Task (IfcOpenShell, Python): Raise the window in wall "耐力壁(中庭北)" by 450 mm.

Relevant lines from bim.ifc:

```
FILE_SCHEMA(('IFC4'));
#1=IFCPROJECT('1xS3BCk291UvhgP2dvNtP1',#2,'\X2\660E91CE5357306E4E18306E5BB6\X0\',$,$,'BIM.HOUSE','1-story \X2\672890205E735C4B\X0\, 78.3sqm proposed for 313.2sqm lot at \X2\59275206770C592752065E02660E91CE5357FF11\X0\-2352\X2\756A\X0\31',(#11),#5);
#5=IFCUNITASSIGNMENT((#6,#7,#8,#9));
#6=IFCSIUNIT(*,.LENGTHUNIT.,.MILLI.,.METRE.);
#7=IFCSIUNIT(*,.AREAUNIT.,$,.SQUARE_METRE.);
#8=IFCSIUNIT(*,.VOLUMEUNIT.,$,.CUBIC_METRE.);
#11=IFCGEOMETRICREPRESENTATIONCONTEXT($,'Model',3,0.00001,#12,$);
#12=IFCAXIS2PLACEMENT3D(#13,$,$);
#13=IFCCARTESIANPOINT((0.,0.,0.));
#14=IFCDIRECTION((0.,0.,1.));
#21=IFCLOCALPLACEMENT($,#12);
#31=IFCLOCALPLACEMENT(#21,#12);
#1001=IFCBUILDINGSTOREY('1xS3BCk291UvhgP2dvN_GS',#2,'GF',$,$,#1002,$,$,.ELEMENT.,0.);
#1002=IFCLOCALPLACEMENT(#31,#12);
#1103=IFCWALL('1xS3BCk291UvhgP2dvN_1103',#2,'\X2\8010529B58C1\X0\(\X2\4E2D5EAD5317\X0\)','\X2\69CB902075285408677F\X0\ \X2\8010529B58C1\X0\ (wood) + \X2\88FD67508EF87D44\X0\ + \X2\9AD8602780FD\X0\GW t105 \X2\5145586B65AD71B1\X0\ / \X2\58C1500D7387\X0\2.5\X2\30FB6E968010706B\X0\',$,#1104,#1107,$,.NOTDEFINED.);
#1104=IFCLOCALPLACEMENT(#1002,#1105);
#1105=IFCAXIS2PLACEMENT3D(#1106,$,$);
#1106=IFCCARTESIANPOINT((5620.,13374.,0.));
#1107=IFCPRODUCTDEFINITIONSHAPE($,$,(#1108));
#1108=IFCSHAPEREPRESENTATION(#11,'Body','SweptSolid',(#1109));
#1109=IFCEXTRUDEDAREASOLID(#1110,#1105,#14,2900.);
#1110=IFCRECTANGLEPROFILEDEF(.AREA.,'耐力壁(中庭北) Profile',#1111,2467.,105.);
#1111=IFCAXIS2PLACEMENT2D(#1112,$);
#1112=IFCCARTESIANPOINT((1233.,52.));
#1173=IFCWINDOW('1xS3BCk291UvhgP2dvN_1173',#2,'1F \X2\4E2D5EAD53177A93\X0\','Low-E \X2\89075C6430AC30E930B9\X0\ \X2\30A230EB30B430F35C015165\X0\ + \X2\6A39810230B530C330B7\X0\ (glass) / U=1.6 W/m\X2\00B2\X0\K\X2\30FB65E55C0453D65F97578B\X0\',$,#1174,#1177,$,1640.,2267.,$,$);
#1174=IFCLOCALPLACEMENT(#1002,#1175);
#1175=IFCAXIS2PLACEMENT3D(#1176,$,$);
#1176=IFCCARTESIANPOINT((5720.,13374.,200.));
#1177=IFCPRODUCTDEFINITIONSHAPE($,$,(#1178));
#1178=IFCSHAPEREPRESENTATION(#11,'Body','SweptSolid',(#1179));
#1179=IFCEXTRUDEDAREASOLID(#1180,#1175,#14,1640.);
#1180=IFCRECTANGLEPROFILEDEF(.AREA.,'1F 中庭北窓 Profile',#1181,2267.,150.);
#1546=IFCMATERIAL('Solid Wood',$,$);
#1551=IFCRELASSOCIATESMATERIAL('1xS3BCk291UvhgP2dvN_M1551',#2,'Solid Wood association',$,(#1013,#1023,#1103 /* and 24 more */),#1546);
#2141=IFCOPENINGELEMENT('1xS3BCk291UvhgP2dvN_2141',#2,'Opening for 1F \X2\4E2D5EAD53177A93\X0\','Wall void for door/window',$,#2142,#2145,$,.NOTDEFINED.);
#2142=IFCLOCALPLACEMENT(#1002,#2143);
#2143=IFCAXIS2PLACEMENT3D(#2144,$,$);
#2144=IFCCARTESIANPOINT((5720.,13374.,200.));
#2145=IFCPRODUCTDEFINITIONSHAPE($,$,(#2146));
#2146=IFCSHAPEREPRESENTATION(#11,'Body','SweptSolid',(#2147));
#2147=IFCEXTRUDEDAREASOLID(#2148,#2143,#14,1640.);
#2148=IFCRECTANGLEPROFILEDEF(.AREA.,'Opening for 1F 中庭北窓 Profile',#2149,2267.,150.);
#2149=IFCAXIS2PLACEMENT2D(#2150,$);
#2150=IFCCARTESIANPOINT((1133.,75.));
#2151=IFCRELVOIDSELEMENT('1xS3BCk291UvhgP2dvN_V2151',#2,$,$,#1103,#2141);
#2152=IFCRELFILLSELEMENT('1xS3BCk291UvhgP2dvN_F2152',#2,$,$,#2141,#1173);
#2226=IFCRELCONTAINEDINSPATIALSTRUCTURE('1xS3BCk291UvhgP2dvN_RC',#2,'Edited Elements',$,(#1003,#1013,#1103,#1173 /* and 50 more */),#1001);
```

```python
import numpy as np
import ifcopenshell
import ifcopenshell.api.geometry
import ifcopenshell.util.placement
import ifcopenshell.util.unit

model = ifcopenshell.open("bim.ifc")
unit_scale = ifcopenshell.util.unit.calculate_unit_scale(model)

window = model.by_guid("1xS3BCk291UvhgP2dvN_1173")
opening = window.FillsVoids[0].RelatingOpeningElement
dz = 0.45 / unit_scale

shift = np.array([0.0, 0.0, dz])
# The window is not placed relative to its opening, so move both.
for product in (opening, window):
    matrix = ifcopenshell.util.placement.get_local_placement(product.ObjectPlacement)
    matrix[:3, 3] += shift
    ifcopenshell.api.geometry.edit_object_placement(model, product=product, matrix=matrix, is_si=False)

print(f"moved by {dz * unit_scale:+.3f} m")

model.write("bim_updated.ifc")
```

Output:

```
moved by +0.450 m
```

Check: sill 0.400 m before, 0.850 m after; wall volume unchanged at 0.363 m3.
